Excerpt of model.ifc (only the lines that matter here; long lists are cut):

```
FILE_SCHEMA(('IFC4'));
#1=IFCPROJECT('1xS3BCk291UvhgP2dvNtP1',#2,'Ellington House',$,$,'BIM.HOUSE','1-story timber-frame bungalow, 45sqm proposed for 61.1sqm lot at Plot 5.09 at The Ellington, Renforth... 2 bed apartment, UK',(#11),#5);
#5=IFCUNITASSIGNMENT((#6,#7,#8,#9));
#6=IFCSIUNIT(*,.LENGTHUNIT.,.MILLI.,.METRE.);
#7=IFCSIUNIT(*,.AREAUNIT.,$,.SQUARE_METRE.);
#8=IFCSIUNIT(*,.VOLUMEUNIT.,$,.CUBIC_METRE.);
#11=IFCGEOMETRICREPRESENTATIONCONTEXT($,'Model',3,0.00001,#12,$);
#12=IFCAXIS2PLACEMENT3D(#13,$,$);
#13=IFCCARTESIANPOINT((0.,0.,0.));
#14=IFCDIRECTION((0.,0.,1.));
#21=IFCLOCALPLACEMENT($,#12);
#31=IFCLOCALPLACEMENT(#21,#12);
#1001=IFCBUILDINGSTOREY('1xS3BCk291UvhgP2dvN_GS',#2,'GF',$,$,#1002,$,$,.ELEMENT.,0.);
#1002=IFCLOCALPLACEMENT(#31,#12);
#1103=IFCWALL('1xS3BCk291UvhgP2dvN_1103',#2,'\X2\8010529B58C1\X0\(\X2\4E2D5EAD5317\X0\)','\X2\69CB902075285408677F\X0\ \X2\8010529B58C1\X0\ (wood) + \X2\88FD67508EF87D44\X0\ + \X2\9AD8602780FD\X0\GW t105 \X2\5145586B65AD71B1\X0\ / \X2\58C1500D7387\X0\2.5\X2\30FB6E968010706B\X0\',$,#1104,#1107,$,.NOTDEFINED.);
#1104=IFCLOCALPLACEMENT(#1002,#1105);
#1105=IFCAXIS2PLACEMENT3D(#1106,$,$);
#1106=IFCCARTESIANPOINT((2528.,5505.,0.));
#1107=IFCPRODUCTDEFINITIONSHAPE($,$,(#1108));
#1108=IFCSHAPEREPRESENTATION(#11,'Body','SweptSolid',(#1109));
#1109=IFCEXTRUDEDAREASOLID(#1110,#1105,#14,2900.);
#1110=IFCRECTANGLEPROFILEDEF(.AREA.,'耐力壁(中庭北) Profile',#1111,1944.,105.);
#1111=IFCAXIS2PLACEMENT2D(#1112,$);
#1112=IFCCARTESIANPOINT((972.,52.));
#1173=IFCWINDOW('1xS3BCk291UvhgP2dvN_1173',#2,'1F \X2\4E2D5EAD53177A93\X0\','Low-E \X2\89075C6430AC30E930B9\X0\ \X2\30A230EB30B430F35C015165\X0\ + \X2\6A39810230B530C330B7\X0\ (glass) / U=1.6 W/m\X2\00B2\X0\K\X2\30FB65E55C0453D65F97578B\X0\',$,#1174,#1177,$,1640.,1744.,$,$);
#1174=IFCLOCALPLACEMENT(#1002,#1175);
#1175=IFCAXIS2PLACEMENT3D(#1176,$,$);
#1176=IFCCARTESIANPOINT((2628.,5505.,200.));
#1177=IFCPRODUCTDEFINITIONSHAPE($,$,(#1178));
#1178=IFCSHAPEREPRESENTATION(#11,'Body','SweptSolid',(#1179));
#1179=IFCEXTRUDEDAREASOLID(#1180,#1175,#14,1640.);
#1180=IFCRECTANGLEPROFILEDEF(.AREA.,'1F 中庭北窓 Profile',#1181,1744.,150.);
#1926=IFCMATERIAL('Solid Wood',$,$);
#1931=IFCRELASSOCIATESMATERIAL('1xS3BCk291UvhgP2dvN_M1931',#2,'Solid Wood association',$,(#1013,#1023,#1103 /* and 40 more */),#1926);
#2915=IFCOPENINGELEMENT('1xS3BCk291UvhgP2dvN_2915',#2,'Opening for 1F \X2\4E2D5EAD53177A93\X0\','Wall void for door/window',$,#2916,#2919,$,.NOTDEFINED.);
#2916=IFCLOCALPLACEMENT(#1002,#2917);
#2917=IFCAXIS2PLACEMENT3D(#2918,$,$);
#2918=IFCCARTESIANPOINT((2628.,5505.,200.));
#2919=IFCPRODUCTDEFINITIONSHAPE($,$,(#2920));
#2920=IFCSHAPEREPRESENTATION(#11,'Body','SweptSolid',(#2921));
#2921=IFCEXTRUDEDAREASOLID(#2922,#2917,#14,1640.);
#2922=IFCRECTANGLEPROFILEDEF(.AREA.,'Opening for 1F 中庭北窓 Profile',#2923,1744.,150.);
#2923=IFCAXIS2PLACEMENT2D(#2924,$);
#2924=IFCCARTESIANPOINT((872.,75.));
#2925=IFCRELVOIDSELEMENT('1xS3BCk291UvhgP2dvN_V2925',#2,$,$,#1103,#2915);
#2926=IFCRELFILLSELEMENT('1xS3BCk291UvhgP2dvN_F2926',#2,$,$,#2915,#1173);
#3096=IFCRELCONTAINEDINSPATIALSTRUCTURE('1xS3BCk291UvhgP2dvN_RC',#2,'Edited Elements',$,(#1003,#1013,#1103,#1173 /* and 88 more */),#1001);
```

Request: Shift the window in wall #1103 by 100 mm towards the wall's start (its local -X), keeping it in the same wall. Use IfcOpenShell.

```python
import ifcopenshell
import ifcopenshell.api.geometry
import ifcopenshell.util.placement
import ifcopenshell.util.unit

model = ifcopenshell.open("model.ifc")
unit_scale = ifcopenshell.util.unit.calculate_unit_scale(model)

window = model.by_guid("1xS3BCk291UvhgP2dvN_1173")
opening = window.FillsVoids[0].RelatingOpeningElement
wall = opening.VoidsElements[0].RelatingBuildingElement

wall_matrix = ifcopenshell.util.placement.get_local_placement(wall.ObjectPlacement)
shift = wall_matrix[:3, 0] * -0.1 / unit_scale
before = ifcopenshell.util.placement.get_local_placement(window.ObjectPlacement)[:3, 3].copy()

# The window is not placed relative to its opening, so move both.
for product in (opening, window):
    matrix = ifcopenshell.util.placement.get_local_placement(product.ObjectPlacement)
    matrix[:3, 3] += shift
    ifcopenshell.api.geometry.edit_object_placement(model, product=product, matrix=matrix, is_si=False)

after = ifcopenshell.util.placement.get_local_placement(window.ObjectPlacement)[:3, 3]
print("window moved by", (after - before).round(3) + 0.0)

model.write("model_updated.ifc")
```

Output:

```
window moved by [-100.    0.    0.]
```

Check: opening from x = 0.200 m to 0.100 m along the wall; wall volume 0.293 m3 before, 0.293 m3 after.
